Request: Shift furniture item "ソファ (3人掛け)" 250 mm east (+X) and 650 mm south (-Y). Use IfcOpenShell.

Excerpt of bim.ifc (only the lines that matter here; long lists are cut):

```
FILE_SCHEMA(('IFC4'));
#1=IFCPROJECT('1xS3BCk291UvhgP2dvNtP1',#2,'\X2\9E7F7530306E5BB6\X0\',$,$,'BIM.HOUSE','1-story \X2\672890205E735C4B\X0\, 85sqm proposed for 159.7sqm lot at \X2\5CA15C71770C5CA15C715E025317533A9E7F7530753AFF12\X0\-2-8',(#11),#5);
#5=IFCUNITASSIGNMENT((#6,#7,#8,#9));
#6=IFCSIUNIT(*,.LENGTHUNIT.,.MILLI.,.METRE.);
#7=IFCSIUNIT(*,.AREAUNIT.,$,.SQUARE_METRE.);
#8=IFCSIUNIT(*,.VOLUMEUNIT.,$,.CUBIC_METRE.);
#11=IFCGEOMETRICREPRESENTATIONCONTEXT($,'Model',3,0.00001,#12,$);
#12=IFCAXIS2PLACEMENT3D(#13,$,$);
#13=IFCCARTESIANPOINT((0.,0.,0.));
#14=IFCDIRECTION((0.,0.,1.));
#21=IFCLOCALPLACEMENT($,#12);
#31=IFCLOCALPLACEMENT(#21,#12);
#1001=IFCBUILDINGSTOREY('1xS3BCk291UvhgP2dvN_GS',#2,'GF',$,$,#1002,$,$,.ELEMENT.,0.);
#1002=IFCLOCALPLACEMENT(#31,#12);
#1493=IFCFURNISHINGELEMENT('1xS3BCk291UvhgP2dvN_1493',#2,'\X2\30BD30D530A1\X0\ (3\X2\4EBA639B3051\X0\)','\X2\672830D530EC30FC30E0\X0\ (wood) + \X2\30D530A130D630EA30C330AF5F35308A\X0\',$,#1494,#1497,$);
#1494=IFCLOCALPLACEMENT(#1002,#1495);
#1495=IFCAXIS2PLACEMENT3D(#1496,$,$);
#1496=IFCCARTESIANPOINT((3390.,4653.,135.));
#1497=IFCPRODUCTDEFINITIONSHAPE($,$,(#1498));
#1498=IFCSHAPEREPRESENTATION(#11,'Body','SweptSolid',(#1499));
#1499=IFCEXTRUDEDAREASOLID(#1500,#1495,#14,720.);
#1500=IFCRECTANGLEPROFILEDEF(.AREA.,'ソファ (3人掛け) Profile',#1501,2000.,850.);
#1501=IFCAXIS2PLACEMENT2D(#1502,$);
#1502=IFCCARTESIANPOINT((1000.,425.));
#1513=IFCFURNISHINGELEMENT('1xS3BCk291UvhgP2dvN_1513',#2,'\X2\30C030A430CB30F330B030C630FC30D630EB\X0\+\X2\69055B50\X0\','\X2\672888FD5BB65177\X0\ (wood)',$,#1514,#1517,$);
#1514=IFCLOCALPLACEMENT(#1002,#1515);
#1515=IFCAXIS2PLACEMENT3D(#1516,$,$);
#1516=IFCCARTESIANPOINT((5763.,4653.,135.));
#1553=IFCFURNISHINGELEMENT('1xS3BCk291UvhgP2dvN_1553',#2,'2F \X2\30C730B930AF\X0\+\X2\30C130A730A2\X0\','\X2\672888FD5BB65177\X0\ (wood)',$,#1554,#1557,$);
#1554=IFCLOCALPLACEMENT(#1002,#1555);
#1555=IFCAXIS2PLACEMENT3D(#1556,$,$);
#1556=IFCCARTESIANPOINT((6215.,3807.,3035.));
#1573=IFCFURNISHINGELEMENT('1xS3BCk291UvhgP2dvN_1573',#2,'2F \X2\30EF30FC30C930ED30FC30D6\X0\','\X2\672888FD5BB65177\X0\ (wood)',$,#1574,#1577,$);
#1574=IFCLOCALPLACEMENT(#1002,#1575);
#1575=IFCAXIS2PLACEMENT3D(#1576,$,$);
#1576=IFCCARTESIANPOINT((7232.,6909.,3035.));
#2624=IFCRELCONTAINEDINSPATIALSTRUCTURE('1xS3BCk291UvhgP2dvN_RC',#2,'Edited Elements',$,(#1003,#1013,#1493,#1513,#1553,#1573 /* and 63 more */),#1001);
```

```python
import ifcopenshell
import ifcopenshell.api.geometry
import ifcopenshell.util.placement

model = ifcopenshell.open("bim.ifc")

item = model.by_guid("1xS3BCk291UvhgP2dvN_1493")
matrix = ifcopenshell.util.placement.get_local_placement(item.ObjectPlacement)
matrix[0, 3] += 250.0
matrix[1, 3] -= 650.0
ifcopenshell.api.geometry.edit_object_placement(model, product=item, matrix=matrix, is_si=False)

print(ifcopenshell.util.placement.get_local_placement(item.ObjectPlacement).round(3) + 0.0)

model.write("bim-out.ifc")
```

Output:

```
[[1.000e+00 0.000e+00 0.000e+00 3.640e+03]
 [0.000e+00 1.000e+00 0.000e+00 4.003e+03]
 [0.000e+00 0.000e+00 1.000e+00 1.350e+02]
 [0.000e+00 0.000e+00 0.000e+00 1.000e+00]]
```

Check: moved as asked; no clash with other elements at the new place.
